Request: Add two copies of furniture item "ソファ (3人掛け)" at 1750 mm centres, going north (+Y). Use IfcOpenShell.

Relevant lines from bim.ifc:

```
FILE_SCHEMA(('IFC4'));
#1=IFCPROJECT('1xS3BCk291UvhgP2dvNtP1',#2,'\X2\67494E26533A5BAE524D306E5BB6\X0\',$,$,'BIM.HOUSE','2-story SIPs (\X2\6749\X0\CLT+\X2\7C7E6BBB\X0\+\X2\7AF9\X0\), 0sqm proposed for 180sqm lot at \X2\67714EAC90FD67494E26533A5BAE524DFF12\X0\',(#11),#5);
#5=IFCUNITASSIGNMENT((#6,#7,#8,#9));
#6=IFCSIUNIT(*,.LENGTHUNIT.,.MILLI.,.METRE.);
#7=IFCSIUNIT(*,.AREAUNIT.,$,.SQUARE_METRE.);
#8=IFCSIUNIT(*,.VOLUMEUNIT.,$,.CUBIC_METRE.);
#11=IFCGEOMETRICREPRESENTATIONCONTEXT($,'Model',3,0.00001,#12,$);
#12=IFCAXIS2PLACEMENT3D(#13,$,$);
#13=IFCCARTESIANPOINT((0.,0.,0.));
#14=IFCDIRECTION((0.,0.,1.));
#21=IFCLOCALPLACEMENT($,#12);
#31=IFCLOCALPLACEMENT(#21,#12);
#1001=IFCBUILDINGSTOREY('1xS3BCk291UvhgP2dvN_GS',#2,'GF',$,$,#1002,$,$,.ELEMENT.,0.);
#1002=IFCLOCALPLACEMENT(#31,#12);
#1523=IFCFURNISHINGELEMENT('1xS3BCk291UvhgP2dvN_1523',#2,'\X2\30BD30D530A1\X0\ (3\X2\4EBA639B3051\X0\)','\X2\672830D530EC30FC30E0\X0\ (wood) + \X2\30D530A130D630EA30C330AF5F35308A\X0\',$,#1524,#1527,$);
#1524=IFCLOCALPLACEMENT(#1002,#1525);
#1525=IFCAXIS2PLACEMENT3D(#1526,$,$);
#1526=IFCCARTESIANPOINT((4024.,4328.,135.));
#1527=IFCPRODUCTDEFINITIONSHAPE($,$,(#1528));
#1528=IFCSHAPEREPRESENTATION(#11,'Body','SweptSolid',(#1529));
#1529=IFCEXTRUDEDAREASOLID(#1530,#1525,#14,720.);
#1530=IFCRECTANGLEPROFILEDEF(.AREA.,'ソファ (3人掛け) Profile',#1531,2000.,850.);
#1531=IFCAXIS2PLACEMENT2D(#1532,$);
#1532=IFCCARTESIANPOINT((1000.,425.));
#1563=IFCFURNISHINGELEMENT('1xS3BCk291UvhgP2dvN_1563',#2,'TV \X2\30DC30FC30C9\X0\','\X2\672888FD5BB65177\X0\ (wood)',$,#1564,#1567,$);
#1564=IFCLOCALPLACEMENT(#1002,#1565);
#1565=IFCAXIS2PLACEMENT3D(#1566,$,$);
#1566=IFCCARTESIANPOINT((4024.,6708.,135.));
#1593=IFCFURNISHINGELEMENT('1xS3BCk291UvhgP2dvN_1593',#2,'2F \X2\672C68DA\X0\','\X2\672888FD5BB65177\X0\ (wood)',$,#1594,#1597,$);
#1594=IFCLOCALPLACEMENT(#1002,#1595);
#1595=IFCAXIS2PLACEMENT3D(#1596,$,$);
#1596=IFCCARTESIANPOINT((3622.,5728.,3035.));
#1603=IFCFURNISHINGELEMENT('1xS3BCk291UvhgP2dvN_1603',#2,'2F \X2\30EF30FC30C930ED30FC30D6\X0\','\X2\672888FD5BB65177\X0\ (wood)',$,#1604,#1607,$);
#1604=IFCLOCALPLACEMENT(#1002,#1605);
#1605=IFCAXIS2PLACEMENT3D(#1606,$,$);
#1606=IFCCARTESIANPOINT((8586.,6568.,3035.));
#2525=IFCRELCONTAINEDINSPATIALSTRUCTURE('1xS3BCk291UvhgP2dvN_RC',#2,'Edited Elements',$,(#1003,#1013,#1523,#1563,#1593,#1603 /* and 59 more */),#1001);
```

```python
import numpy as np
import ifcopenshell
import ifcopenshell.api.geometry
import ifcopenshell.api.root
import ifcopenshell.util.element
import ifcopenshell.util.placement
import ifcopenshell.util.unit

model = ifcopenshell.open("bim.ifc")
unit_scale = ifcopenshell.util.unit.calculate_unit_scale(model)


def reuse_history(source, copy):
    """copy_class also copies each property set's owner history, people and application; keep the originals."""
    for rel in copy.IsDefinedBy:
        if rel.is_a("IfcRelDefinesByProperties") and (history := rel.RelatingPropertyDefinition.OwnerHistory):
            rel.RelatingPropertyDefinition.OwnerHistory = source.OwnerHistory
            ifcopenshell.util.element.remove_deep2(model, history)


source = model.by_id(1523)
base = ifcopenshell.util.placement.get_local_placement(source.ObjectPlacement)
step = np.array([0.0, 1.0, 0.0]) * 1.75 / unit_scale

for i in range(1, 3):
    copy = ifcopenshell.api.root.copy_class(model, product=source)
    copy.Representation = ifcopenshell.util.element.copy_deep(
        model, source.Representation, exclude=["IfcGeometricRepresentationContext", "IfcRepresentationMap"]
    )
    reuse_history(source, copy)
    matrix = base.copy()
    matrix[:3, 3] += i * step
    print("added at", matrix[:3, 3].round(3) + 0.0)
    ifcopenshell.api.geometry.edit_object_placement(model, product=copy, matrix=matrix, is_si=False)

model.write("bim_edited.ifc")
```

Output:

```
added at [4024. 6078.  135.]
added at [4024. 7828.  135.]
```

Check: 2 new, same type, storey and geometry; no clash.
